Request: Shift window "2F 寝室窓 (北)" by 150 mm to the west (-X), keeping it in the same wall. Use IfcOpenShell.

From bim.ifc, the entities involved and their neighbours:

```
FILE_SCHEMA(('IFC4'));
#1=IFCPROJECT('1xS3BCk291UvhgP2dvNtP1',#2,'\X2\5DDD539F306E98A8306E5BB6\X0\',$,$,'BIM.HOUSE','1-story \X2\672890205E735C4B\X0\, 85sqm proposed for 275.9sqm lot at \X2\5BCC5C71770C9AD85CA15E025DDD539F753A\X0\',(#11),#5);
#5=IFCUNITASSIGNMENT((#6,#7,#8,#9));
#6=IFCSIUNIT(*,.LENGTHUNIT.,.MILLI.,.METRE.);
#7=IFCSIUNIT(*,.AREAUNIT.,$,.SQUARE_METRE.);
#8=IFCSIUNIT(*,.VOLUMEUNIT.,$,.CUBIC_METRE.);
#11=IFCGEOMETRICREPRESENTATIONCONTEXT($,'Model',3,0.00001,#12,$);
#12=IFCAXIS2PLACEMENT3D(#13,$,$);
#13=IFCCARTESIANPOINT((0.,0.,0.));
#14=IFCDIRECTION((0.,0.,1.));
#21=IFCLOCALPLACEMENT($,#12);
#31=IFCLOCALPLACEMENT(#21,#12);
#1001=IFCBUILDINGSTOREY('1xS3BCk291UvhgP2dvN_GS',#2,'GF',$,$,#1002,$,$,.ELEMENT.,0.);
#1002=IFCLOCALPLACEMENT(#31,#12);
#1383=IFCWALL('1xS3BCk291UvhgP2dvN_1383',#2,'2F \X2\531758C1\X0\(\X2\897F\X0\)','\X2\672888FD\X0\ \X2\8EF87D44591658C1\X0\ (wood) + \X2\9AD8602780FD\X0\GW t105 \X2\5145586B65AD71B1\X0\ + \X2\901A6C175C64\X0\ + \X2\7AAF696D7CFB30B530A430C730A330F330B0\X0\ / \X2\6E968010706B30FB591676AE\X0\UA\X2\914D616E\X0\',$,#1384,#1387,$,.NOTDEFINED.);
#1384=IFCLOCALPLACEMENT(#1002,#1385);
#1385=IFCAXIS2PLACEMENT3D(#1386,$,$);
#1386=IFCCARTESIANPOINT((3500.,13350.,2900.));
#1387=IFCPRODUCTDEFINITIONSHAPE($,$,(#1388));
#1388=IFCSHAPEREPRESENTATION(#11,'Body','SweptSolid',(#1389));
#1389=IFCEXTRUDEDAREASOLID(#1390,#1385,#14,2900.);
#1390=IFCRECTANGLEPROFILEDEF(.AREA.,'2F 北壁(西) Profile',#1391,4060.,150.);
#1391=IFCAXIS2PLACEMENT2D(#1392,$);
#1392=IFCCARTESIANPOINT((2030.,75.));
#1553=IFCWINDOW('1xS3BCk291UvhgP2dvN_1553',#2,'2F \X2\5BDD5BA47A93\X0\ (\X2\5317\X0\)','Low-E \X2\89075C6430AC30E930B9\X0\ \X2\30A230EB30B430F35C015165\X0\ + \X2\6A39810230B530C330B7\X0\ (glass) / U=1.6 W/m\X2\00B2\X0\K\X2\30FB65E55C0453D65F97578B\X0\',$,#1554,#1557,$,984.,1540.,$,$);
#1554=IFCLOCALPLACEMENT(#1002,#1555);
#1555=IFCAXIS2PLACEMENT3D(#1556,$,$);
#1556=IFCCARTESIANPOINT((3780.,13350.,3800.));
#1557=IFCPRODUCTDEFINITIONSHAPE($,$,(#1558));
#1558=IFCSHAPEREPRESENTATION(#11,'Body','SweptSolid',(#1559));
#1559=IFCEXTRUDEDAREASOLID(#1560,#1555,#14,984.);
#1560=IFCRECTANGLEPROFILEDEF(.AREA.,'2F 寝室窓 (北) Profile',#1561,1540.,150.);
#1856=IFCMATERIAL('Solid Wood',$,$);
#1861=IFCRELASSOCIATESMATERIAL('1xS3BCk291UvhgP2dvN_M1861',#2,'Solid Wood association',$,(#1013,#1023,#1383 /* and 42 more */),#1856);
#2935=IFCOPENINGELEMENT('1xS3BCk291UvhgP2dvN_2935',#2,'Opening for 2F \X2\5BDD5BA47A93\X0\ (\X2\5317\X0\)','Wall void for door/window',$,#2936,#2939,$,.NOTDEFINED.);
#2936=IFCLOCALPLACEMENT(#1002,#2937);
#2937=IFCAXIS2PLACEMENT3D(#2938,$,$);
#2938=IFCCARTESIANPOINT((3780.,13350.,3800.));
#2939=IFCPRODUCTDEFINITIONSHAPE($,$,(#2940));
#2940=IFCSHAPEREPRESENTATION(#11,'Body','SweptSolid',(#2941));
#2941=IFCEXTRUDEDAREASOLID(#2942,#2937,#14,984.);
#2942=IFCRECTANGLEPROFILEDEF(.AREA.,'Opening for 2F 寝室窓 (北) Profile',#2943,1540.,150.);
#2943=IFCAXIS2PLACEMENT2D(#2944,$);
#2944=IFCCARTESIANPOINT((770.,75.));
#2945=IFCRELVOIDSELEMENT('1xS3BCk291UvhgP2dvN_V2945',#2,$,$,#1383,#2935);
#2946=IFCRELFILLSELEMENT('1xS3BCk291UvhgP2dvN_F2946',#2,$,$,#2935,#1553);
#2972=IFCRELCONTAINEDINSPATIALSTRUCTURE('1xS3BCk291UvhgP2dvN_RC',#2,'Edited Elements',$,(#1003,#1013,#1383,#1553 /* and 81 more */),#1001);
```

```python
import ifcopenshell
import ifcopenshell.api.geometry
import ifcopenshell.util.placement
import ifcopenshell.util.unit

model = ifcopenshell.open("bim.ifc")
unit_scale = ifcopenshell.util.unit.calculate_unit_scale(model)

window = model.by_guid("1xS3BCk291UvhgP2dvN_1553")
opening = window.FillsVoids[0].RelatingOpeningElement
wall = opening.VoidsElements[0].RelatingBuildingElement

wall_matrix = ifcopenshell.util.placement.get_local_placement(wall.ObjectPlacement)
shift = wall_matrix[:3, 0] * -0.15 / unit_scale
before = ifcopenshell.util.placement.get_local_placement(window.ObjectPlacement)[:3, 3].copy()

# The window is not placed relative to its opening, so move both.
for product in (opening, window):
    matrix = ifcopenshell.util.placement.get_local_placement(product.ObjectPlacement)
    matrix[:3, 3] += shift
    ifcopenshell.api.geometry.edit_object_placement(model, product=product, matrix=matrix, is_si=False)

after = ifcopenshell.util.placement.get_local_placement(window.ObjectPlacement)[:3, 3]
print("window moved by", (after - before).round(3) + 0.0)

model.write("bim_edited.ifc")
```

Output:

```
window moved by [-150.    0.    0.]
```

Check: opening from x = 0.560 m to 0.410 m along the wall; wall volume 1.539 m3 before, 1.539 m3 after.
